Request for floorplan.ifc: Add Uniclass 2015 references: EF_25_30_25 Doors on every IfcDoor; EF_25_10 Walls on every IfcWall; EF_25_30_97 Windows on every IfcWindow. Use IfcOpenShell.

First a look at what the model holds.

```python
import ifcopenshell

model = ifcopenshell.open("floorplan.ifc")
print(model.schema)
print("classifications:", [c.Name for c in model.by_type("IfcClassification")])
for ifc_class in ("IfcDoor", "IfcRoof", "IfcStair", "IfcWall", "IfcWindow"):
    print(ifc_class, len(model.by_type(ifc_class)))
```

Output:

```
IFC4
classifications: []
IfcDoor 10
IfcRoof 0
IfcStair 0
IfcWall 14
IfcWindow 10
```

```python
import ifcopenshell
import ifcopenshell.api.classification

model = ifcopenshell.open("floorplan.ifc")

system = ifcopenshell.api.classification.add_classification(model, classification="Uniclass 2015")

codes = {
    "IfcDoor": ("EF_25_30_25", "Doors"),
    "IfcWall": ("EF_25_10", "Walls"),
    "IfcWindow": ("EF_25_30_97", "Windows"),
}
for ifc_class, (code, name) in codes.items():
    products = model.by_type(ifc_class)
    ifcopenshell.api.classification.add_reference(
        model, products=products, classification=system, identification=code, name=name
    )
    print(code, len(products))

model.write("floorplan_edited.ifc")
```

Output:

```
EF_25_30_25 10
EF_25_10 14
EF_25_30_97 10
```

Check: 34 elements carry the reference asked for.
